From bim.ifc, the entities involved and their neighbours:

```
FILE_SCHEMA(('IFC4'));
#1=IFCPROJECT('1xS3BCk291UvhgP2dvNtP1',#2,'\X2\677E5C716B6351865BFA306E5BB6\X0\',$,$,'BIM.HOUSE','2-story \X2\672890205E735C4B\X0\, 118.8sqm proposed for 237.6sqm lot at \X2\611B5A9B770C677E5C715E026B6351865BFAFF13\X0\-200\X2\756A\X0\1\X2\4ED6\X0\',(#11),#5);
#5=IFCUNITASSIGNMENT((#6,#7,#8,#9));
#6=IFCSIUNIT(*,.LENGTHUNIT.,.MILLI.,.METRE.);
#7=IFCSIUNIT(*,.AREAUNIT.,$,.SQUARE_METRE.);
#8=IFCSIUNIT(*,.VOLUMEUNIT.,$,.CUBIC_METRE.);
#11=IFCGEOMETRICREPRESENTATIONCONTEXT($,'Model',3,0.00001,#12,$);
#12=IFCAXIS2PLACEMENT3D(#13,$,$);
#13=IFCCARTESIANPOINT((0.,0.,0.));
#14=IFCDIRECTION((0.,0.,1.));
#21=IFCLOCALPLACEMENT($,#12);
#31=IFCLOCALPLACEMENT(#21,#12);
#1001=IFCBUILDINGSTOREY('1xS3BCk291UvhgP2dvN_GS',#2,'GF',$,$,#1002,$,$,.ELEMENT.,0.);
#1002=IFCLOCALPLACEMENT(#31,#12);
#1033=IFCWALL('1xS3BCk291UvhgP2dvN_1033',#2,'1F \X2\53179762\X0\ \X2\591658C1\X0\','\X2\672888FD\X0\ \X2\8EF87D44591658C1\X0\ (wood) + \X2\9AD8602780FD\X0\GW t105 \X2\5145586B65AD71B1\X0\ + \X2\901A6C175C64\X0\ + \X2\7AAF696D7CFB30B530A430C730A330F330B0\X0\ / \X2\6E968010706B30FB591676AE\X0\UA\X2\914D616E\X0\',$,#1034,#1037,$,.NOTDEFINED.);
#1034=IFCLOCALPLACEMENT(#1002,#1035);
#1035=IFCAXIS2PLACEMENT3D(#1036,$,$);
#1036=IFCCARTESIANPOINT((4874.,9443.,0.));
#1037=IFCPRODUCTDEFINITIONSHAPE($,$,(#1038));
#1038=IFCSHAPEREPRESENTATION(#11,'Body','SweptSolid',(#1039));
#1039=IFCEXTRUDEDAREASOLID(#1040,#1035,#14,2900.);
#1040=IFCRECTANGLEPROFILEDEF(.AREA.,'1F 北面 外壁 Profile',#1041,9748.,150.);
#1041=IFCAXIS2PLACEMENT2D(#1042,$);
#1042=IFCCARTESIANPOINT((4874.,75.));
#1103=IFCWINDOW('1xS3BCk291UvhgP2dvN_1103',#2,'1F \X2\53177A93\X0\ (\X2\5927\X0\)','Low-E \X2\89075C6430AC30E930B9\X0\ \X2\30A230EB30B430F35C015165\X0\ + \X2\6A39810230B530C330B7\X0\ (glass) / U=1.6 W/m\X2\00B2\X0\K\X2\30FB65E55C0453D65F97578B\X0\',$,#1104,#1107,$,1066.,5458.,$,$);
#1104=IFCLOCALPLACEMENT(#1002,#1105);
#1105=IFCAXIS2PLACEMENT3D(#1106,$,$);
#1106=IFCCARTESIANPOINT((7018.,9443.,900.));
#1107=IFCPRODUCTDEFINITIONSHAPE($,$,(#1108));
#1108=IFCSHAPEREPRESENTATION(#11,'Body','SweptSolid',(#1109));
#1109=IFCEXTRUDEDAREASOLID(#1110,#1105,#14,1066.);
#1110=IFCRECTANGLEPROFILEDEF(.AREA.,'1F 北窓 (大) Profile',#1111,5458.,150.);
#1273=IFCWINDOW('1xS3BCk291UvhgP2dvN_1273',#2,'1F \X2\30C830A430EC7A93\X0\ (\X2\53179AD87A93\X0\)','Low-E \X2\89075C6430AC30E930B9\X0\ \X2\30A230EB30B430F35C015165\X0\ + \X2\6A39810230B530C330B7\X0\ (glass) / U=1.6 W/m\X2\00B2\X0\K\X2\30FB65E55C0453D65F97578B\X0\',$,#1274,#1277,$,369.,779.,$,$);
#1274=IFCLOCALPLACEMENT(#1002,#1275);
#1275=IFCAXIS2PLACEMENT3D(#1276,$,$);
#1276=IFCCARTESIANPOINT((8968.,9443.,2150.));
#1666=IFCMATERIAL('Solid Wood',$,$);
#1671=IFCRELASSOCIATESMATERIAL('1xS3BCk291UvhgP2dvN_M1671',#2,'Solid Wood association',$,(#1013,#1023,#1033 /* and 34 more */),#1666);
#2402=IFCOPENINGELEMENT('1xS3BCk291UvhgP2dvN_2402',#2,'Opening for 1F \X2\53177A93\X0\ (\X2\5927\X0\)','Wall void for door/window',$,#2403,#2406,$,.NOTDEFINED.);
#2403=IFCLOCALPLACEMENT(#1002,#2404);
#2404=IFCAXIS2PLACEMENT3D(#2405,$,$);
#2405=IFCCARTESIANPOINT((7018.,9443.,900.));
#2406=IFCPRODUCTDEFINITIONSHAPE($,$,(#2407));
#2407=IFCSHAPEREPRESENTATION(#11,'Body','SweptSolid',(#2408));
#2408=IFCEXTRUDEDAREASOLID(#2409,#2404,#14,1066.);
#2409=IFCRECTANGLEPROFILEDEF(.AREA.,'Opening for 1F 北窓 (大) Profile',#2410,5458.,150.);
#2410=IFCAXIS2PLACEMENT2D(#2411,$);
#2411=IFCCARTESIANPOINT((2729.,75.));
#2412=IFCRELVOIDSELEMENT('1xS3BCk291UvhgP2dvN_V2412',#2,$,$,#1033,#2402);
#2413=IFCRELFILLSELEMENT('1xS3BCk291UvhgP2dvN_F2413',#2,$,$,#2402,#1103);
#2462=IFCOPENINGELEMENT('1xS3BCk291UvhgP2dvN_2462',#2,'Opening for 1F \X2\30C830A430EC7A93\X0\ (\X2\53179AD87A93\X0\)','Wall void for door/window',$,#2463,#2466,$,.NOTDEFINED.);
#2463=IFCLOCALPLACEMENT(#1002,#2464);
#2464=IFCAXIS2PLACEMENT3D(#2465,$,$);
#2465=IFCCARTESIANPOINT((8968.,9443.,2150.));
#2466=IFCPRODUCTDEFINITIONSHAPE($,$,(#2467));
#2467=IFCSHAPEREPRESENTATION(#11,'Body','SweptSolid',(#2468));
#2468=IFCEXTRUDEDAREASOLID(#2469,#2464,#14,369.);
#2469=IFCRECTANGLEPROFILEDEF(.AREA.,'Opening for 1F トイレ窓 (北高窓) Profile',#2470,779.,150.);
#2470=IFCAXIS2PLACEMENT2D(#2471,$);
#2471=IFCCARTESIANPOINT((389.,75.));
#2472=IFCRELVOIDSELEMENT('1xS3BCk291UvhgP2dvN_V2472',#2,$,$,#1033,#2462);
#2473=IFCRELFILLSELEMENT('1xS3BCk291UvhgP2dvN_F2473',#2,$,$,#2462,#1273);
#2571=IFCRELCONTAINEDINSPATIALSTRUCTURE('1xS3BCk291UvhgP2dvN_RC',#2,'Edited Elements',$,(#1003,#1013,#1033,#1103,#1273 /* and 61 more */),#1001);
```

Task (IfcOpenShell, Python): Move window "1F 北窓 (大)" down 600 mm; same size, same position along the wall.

```python
import numpy as np
import ifcopenshell
import ifcopenshell.api.geometry
import ifcopenshell.util.placement
import ifcopenshell.util.unit

model = ifcopenshell.open("bim.ifc")
unit_scale = ifcopenshell.util.unit.calculate_unit_scale(model)

window = model.by_id(1103)
opening = window.FillsVoids[0].RelatingOpeningElement
dz = -0.6 / unit_scale

shift = np.array([0.0, 0.0, dz])
# The window is not placed relative to its opening, so move both.
for product in (opening, window):
    matrix = ifcopenshell.util.placement.get_local_placement(product.ObjectPlacement)
    matrix[:3, 3] += shift
    ifcopenshell.api.geometry.edit_object_placement(model, product=product, matrix=matrix, is_si=False)

print(f"moved by {dz * unit_scale:+.3f} m")

model.write("bim_updated.ifc")
```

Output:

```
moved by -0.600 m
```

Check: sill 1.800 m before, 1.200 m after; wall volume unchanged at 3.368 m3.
